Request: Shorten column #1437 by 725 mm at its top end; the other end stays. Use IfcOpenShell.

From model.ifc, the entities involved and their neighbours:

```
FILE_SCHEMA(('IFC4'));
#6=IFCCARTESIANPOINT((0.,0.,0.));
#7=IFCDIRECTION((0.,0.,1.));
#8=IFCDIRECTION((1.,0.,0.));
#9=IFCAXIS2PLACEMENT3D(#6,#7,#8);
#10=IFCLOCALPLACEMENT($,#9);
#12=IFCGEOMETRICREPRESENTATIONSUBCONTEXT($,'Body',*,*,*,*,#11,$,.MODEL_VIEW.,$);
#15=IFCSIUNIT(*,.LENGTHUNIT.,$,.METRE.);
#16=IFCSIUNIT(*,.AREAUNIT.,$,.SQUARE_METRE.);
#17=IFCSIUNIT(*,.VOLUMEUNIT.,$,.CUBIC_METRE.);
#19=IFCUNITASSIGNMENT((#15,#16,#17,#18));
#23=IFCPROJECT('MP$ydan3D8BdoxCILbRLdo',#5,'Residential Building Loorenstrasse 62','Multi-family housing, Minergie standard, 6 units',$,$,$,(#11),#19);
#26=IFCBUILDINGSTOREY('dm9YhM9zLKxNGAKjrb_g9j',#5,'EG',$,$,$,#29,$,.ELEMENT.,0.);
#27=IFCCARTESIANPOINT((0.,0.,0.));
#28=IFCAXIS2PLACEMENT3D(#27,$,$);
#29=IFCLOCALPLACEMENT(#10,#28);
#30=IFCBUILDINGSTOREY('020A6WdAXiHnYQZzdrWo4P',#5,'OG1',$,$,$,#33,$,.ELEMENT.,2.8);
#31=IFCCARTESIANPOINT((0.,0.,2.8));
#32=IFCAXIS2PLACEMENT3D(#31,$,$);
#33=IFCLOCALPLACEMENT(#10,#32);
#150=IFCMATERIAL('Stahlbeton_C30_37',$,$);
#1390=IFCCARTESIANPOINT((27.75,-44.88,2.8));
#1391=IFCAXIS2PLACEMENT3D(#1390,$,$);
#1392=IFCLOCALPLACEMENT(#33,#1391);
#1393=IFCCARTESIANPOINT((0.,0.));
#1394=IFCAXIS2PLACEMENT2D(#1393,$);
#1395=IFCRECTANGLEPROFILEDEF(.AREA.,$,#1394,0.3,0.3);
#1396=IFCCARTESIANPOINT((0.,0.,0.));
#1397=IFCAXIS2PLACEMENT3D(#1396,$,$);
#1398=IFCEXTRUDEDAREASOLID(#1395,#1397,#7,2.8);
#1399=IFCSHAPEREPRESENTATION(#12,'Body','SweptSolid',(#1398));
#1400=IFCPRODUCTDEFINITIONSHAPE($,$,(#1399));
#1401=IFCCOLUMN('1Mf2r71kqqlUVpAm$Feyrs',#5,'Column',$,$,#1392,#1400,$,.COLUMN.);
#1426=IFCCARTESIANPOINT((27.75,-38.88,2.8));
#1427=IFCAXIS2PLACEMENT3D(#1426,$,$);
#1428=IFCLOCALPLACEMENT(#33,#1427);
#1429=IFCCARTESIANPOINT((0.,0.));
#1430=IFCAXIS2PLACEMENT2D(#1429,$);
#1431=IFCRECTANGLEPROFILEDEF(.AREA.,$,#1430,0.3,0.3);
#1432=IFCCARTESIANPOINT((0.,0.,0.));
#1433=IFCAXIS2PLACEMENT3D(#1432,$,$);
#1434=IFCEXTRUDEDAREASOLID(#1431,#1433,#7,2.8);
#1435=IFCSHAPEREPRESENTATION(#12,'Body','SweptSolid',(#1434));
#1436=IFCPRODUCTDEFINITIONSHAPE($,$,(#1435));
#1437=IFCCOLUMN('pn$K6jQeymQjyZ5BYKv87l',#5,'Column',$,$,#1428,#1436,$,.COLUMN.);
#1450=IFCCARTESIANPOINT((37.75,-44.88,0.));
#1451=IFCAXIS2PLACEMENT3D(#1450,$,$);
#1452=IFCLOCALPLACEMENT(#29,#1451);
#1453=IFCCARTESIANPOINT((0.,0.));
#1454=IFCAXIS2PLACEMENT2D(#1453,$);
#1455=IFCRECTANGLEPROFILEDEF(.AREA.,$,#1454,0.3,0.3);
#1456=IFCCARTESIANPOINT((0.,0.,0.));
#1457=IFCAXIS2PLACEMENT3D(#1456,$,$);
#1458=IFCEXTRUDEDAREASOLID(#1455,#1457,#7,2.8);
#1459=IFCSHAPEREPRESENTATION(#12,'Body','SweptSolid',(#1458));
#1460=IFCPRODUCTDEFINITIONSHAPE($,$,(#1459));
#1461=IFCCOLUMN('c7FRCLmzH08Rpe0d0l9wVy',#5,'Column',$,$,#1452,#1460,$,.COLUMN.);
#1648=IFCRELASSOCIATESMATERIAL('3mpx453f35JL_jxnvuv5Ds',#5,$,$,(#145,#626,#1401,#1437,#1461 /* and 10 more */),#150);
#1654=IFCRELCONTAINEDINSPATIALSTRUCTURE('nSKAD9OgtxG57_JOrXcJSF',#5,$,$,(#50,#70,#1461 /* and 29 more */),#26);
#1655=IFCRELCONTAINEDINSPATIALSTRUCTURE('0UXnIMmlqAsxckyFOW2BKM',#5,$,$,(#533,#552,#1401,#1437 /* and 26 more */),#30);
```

```python
import ifcopenshell

model = ifcopenshell.open("model.ifc")

member = model.by_guid("pn$K6jQeymQjyZ5BYKv87l")
change = -0.725

# The extrusion runs towards the end named, so only its depth changes.
body = next(r for r in member.Representation.Representations if r.RepresentationIdentifier == "Body")
solid = body.Items[0]
old_length = solid.Depth
solid.Depth += change

print(f"length {old_length:g} -> {solid.Depth:g}")

model.write("model_rev.ifc")
```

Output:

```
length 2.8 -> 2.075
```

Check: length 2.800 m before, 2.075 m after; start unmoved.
